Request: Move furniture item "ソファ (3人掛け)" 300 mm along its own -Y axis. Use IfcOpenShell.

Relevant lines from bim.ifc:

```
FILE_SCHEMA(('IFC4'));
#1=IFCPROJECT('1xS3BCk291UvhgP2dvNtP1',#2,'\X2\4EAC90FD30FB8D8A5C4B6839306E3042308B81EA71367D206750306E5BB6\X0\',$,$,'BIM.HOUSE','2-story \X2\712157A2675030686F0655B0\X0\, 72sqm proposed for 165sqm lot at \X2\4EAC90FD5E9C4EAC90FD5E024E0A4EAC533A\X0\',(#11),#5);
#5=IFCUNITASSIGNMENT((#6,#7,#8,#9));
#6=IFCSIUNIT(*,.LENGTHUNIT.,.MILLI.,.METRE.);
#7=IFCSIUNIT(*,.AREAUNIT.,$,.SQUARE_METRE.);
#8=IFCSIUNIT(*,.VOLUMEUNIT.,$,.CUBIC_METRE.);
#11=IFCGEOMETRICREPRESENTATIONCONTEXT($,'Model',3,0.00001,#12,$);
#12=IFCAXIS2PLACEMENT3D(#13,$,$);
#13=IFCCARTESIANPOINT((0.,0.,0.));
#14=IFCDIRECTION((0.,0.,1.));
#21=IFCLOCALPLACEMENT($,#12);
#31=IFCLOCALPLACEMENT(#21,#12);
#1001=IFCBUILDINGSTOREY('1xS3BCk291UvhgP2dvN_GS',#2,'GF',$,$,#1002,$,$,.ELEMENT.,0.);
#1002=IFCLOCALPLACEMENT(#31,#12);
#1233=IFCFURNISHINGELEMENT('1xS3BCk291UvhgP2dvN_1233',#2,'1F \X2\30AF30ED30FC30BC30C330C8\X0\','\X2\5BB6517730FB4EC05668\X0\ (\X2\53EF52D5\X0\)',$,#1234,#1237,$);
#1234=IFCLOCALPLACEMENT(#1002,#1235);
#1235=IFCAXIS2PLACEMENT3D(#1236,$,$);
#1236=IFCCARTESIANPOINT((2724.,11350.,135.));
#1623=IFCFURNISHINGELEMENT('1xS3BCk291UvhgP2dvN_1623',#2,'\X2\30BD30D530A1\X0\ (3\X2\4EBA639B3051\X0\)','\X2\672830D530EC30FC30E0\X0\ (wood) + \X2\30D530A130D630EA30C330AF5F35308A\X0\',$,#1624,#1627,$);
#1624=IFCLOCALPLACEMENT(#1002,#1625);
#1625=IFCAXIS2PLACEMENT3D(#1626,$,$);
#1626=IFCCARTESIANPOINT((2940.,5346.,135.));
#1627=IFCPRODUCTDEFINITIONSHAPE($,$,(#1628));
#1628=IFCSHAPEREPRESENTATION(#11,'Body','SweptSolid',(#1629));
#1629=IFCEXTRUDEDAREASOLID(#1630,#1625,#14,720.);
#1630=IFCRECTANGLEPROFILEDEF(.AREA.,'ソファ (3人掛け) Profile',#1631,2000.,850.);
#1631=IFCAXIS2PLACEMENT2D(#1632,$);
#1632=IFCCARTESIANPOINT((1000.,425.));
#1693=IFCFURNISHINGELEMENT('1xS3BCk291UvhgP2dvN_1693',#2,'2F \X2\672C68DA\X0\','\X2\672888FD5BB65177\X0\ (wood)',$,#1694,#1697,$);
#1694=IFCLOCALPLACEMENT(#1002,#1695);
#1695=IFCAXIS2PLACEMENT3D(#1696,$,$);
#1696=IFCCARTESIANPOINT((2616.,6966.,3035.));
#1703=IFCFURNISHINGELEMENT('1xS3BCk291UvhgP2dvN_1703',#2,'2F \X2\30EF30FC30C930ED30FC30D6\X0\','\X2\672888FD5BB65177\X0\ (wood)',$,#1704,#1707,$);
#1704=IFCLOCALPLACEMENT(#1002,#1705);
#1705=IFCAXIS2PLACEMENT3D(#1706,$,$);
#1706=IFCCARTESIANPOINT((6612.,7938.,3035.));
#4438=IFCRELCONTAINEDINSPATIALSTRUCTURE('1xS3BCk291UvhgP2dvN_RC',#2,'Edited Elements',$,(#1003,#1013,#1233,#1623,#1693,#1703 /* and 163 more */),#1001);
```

```python
import ifcopenshell
import ifcopenshell.api.geometry
import ifcopenshell.util.placement
import ifcopenshell.util.unit

model = ifcopenshell.open("bim.ifc")
unit_scale = ifcopenshell.util.unit.calculate_unit_scale(model)

item = model.by_id(1623)
matrix = ifcopenshell.util.placement.get_local_placement(item.ObjectPlacement)
matrix[:3, 3] -= matrix[:3, 1] * 0.3 / unit_scale
ifcopenshell.api.geometry.edit_object_placement(model, product=item, matrix=matrix, is_si=False)

print(ifcopenshell.util.placement.get_local_placement(item.ObjectPlacement).round(3) + 0.0)

model.write("bim_edited.ifc")
```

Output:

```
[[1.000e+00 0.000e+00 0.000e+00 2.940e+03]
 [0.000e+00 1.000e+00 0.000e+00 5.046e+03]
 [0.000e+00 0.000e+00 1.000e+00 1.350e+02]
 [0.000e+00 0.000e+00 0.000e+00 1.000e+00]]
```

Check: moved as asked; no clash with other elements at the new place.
